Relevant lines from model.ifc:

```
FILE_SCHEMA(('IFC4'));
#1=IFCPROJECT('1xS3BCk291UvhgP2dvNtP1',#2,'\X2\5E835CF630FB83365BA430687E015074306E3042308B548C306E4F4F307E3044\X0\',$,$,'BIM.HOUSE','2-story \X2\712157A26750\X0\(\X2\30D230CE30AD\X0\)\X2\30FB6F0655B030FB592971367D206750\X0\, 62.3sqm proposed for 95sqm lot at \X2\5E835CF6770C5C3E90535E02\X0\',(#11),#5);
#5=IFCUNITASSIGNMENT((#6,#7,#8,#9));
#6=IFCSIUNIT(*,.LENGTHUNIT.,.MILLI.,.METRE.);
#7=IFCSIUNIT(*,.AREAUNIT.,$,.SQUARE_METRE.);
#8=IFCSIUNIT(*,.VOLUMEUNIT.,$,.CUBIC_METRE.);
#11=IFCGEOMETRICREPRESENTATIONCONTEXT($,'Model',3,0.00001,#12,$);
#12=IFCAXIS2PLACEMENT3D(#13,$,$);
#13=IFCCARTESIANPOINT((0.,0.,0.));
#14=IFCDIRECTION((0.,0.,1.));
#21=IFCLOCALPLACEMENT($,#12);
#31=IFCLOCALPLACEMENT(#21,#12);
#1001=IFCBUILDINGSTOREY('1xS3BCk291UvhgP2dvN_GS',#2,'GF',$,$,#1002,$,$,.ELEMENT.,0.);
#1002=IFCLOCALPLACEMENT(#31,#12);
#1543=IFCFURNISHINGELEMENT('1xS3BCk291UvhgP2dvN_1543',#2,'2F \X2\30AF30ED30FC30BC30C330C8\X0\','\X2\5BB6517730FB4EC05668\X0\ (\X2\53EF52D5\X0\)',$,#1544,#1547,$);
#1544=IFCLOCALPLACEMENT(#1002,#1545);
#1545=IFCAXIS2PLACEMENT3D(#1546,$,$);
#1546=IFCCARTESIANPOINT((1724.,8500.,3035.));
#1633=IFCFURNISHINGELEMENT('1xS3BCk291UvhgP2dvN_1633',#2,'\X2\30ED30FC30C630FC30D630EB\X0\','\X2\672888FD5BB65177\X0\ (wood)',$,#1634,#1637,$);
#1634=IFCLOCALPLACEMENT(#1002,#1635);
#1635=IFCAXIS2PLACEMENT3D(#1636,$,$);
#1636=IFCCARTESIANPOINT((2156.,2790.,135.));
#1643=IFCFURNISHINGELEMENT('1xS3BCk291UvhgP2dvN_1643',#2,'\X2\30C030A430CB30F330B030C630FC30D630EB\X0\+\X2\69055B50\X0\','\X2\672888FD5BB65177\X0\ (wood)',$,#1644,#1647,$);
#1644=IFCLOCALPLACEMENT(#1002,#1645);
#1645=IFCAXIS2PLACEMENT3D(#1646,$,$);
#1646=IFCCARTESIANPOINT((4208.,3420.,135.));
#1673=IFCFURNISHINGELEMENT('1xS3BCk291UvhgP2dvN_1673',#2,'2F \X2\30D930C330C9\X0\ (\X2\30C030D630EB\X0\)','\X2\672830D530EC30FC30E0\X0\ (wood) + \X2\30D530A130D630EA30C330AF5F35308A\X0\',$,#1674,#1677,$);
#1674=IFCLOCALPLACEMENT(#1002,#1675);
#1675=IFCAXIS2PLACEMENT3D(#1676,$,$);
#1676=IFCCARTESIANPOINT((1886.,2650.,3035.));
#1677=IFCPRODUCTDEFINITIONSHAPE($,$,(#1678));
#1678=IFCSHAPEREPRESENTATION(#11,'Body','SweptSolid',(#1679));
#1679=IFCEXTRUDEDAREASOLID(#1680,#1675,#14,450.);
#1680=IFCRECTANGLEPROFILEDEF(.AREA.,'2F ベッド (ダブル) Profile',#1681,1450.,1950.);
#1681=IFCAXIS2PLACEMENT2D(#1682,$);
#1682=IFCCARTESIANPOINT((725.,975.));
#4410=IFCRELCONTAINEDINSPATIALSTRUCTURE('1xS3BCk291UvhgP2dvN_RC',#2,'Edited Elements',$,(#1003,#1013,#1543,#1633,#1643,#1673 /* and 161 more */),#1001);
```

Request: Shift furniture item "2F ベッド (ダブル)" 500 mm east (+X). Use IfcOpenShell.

```python
import ifcopenshell
import ifcopenshell.api.geometry
import ifcopenshell.util.placement

model = ifcopenshell.open("model.ifc")

item = model.by_guid("1xS3BCk291UvhgP2dvN_1673")
matrix = ifcopenshell.util.placement.get_local_placement(item.ObjectPlacement)
matrix[0, 3] += 500.0
ifcopenshell.api.geometry.edit_object_placement(model, product=item, matrix=matrix, is_si=False)

print(ifcopenshell.util.placement.get_local_placement(item.ObjectPlacement).round(3) + 0.0)

model.write("model_edited.ifc")
```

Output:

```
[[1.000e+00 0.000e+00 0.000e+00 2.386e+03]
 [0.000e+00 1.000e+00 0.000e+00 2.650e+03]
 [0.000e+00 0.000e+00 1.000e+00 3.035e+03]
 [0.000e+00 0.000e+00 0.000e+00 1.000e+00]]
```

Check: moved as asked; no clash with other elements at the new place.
